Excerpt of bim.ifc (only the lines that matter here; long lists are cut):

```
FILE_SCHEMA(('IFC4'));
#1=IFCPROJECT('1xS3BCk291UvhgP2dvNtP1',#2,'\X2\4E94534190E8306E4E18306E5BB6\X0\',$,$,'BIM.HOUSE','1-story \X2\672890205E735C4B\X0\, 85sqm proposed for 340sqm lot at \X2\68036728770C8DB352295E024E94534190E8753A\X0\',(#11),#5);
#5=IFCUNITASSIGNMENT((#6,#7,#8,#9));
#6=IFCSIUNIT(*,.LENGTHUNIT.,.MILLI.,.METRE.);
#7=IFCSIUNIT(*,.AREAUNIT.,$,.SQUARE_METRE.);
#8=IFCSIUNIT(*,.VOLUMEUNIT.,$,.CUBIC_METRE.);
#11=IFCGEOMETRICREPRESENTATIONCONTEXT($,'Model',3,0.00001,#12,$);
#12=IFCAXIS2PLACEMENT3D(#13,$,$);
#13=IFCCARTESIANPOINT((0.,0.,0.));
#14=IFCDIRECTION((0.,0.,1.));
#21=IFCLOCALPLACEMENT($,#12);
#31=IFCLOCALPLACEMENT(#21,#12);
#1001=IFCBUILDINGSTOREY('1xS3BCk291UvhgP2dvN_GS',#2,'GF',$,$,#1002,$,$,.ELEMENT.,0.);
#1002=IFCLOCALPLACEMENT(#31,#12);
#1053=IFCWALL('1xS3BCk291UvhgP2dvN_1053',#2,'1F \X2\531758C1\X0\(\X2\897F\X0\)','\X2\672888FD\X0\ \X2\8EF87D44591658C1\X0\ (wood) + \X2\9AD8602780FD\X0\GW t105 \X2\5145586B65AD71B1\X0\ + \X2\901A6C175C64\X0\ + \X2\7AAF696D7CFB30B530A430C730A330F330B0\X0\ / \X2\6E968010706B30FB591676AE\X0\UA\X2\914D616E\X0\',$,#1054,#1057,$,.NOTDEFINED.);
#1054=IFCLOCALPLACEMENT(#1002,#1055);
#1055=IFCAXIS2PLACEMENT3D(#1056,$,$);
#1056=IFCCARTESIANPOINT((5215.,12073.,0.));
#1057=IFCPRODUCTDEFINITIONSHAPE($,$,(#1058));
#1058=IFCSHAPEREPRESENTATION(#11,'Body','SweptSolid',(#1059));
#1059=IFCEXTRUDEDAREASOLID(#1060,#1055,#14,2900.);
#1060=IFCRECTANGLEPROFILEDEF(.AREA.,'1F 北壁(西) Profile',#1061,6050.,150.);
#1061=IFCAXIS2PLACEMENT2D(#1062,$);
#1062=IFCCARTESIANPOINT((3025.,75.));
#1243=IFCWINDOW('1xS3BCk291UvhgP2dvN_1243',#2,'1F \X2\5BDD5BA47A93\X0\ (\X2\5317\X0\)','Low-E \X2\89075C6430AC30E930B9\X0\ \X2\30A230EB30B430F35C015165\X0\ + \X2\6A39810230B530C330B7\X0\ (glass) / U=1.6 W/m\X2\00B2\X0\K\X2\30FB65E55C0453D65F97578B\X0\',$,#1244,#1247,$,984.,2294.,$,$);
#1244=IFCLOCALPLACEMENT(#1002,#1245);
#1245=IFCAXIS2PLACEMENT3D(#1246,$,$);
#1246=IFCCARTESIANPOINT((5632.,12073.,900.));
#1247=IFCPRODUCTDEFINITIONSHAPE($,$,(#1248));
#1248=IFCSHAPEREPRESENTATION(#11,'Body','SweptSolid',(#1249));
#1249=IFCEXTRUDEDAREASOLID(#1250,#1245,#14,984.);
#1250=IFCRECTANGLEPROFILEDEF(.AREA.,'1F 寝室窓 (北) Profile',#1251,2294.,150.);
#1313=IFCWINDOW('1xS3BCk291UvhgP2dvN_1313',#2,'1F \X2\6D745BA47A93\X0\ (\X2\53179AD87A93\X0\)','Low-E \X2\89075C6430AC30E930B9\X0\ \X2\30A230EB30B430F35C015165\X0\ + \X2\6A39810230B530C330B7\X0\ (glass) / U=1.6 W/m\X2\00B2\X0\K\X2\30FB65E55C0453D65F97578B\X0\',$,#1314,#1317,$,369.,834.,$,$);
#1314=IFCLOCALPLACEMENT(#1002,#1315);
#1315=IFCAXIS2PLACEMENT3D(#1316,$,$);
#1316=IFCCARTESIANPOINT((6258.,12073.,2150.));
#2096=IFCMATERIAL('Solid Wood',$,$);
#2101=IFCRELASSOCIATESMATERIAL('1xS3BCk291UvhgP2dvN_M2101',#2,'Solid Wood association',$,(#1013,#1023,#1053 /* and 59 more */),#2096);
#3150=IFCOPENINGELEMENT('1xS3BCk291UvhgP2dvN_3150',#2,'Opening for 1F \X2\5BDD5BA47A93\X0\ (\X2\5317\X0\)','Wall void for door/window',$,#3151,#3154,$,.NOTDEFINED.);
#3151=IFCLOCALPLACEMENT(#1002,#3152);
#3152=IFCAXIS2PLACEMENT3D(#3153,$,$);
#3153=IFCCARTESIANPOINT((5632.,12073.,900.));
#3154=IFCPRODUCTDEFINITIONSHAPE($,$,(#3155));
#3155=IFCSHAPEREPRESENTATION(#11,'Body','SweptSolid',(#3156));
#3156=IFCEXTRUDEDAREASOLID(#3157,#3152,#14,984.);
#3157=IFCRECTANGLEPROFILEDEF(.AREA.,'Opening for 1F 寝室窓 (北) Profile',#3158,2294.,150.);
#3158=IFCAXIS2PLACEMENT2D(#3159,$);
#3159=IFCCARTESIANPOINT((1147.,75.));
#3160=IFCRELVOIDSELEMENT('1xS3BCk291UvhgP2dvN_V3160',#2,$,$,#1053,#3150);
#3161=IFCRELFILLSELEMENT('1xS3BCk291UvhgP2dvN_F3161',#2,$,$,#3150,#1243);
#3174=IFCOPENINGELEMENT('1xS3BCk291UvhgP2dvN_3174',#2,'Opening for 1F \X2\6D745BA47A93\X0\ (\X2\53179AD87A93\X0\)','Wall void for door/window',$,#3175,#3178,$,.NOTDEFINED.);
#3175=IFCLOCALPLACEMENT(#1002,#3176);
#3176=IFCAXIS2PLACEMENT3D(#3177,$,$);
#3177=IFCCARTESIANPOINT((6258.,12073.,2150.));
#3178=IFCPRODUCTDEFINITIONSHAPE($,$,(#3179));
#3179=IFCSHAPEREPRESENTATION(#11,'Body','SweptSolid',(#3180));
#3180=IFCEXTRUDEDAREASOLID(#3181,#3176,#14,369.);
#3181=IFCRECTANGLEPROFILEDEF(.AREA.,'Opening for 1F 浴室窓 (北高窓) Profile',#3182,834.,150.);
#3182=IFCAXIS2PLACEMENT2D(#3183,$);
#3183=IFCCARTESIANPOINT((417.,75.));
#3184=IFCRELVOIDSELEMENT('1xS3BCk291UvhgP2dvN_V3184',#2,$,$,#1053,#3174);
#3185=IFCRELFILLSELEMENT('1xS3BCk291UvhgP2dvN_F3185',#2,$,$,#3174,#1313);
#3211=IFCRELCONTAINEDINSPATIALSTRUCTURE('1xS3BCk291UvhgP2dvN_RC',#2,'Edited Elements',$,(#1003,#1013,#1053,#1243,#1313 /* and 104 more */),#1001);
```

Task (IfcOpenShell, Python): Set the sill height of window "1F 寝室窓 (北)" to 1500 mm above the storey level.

```python
import numpy as np
import ifcopenshell
import ifcopenshell.api.geometry
import ifcopenshell.geom
import ifcopenshell.util.element
import ifcopenshell.util.placement
import ifcopenshell.util.shape
import ifcopenshell.util.unit

model = ifcopenshell.open("bim.ifc")
unit_scale = ifcopenshell.util.unit.calculate_unit_scale(model)

window = model.by_guid("1xS3BCk291UvhgP2dvN_1243")
opening = window.FillsVoids[0].RelatingOpeningElement
storey = ifcopenshell.util.element.get_container(window, ifc_class="IfcBuildingStorey")
level = ifcopenshell.util.placement.get_local_placement(storey.ObjectPlacement)[2, 3]

# The opening's origin need not be at the sill, so measure its lowest point.
shape = ifcopenshell.geom.create_shape(ifcopenshell.geom.settings(), opening)
bottom = ifcopenshell.util.shape.get_shape_bottom_elevation(shape, shape.geometry) / unit_scale
dz = level + 1.5 / unit_scale - bottom

shift = np.array([0.0, 0.0, dz])
# The window is not placed relative to its opening, so move both.
for product in (opening, window):
    matrix = ifcopenshell.util.placement.get_local_placement(product.ObjectPlacement)
    matrix[:3, 3] += shift
    ifcopenshell.api.geometry.edit_object_placement(model, product=product, matrix=matrix, is_si=False)

print(f"moved by {dz * unit_scale:+.3f} m")

model.write("bim_v2.ifc")
```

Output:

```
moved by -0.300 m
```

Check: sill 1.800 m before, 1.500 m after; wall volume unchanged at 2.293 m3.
